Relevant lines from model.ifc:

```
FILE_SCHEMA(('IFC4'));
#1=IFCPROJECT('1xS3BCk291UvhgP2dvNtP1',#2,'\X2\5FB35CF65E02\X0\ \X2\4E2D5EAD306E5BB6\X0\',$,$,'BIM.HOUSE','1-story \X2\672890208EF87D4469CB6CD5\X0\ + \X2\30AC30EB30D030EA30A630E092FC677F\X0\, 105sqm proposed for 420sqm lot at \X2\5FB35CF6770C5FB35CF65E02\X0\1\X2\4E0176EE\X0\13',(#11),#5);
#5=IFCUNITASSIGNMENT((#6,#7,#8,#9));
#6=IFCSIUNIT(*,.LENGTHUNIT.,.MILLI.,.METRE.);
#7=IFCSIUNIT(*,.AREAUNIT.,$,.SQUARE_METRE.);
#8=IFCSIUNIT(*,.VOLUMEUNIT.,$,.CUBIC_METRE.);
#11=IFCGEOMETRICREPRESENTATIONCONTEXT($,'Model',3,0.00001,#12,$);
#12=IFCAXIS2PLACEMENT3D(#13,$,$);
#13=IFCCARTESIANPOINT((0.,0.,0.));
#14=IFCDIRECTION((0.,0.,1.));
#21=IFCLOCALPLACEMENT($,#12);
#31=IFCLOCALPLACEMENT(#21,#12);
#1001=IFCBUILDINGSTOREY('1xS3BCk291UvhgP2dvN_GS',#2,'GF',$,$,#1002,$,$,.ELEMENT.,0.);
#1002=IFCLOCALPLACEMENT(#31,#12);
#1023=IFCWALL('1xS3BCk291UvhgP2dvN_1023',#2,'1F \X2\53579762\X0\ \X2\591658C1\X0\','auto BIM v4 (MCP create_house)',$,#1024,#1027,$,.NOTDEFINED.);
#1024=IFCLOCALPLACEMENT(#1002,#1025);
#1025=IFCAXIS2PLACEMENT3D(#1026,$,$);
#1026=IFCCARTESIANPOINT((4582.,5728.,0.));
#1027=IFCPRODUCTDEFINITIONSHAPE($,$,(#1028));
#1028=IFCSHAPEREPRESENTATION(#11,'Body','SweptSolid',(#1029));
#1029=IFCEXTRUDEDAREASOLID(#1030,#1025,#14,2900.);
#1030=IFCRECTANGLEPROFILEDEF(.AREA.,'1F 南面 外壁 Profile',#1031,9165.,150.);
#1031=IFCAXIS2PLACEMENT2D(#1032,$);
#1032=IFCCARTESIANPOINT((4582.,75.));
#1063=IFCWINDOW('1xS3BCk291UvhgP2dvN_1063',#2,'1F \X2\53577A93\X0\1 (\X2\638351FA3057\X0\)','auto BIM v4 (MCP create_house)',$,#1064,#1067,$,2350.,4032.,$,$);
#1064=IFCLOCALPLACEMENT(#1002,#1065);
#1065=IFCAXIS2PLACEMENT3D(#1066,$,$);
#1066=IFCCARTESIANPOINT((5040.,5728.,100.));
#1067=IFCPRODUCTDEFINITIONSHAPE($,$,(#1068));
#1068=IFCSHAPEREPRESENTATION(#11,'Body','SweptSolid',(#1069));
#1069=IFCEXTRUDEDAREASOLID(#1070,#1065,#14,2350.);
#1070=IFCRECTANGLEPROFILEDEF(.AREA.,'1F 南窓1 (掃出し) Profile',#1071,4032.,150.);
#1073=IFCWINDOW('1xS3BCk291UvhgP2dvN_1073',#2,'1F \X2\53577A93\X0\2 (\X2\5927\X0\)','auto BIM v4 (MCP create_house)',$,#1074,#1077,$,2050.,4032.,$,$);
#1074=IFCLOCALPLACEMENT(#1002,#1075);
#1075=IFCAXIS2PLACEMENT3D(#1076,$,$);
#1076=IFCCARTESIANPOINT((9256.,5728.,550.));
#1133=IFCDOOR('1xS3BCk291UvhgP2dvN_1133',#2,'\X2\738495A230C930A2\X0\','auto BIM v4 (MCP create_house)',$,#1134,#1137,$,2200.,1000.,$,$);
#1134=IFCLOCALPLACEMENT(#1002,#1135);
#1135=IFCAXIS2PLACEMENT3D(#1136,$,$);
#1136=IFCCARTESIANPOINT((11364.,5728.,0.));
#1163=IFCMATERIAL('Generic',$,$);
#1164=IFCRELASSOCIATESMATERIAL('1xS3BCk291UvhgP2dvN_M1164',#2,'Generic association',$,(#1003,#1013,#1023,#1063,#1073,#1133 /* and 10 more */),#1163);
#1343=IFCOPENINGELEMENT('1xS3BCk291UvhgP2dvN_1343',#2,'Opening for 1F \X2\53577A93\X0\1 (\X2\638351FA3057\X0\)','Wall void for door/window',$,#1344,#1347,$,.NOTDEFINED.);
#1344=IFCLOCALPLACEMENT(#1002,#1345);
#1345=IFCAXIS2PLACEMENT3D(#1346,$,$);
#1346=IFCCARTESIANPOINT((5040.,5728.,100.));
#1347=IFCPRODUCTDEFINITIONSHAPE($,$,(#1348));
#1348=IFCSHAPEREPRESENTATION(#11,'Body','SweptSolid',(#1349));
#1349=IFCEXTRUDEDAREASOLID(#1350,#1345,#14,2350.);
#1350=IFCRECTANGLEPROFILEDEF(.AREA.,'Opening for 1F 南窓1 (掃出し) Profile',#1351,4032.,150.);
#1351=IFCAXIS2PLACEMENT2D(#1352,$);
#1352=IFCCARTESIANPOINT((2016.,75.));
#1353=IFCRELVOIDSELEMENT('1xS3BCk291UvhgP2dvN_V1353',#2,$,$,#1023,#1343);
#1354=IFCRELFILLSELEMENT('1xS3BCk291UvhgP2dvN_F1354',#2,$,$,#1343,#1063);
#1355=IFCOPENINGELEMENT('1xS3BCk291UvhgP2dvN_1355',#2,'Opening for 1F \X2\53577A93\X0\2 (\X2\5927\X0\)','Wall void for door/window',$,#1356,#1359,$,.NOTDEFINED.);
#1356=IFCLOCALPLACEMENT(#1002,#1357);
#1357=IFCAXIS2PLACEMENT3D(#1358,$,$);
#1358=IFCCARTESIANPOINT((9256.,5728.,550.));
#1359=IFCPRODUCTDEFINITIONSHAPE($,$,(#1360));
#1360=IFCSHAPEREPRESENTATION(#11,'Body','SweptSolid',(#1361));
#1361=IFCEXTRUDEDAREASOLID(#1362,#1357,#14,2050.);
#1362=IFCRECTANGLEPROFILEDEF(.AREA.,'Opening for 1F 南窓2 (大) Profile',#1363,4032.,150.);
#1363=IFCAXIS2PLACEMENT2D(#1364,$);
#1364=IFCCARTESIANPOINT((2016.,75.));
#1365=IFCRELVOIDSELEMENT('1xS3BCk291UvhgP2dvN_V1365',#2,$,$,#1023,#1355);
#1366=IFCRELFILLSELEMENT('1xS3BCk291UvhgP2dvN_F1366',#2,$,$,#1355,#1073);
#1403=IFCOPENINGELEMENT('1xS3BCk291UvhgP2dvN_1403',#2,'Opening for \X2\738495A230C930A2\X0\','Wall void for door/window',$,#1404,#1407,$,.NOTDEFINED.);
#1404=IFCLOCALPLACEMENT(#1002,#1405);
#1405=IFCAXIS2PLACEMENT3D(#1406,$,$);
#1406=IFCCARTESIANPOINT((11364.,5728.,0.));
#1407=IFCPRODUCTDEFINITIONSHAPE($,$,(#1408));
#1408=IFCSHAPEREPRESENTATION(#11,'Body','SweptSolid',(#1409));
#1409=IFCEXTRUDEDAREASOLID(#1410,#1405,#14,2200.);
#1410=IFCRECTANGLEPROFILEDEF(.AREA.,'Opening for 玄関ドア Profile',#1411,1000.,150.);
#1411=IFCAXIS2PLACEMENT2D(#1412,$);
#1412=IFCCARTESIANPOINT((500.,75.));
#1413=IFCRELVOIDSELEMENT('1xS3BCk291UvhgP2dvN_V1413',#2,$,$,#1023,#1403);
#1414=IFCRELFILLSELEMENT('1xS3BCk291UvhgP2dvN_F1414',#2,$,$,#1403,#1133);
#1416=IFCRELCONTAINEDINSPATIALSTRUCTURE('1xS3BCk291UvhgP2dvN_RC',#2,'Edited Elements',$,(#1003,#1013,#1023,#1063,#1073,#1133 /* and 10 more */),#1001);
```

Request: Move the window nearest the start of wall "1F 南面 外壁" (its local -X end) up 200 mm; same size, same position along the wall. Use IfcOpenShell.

```python
import numpy as np
import ifcopenshell
import ifcopenshell.api.geometry
import ifcopenshell.util.placement
import ifcopenshell.util.unit

model = ifcopenshell.open("model.ifc")
unit_scale = ifcopenshell.util.unit.calculate_unit_scale(model)

window = model.by_id(1063)
opening = window.FillsVoids[0].RelatingOpeningElement
dz = 0.2 / unit_scale

shift = np.array([0.0, 0.0, dz])
# The window is not placed relative to its opening, so move both.
for product in (opening, window):
    matrix = ifcopenshell.util.placement.get_local_placement(product.ObjectPlacement)
    matrix[:3, 3] += shift
    ifcopenshell.api.geometry.edit_object_placement(model, product=product, matrix=matrix, is_si=False)

print(f"moved by {dz * unit_scale:+.3f} m")

model.write("model-out.ifc")
```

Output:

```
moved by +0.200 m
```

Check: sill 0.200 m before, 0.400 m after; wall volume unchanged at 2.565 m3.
